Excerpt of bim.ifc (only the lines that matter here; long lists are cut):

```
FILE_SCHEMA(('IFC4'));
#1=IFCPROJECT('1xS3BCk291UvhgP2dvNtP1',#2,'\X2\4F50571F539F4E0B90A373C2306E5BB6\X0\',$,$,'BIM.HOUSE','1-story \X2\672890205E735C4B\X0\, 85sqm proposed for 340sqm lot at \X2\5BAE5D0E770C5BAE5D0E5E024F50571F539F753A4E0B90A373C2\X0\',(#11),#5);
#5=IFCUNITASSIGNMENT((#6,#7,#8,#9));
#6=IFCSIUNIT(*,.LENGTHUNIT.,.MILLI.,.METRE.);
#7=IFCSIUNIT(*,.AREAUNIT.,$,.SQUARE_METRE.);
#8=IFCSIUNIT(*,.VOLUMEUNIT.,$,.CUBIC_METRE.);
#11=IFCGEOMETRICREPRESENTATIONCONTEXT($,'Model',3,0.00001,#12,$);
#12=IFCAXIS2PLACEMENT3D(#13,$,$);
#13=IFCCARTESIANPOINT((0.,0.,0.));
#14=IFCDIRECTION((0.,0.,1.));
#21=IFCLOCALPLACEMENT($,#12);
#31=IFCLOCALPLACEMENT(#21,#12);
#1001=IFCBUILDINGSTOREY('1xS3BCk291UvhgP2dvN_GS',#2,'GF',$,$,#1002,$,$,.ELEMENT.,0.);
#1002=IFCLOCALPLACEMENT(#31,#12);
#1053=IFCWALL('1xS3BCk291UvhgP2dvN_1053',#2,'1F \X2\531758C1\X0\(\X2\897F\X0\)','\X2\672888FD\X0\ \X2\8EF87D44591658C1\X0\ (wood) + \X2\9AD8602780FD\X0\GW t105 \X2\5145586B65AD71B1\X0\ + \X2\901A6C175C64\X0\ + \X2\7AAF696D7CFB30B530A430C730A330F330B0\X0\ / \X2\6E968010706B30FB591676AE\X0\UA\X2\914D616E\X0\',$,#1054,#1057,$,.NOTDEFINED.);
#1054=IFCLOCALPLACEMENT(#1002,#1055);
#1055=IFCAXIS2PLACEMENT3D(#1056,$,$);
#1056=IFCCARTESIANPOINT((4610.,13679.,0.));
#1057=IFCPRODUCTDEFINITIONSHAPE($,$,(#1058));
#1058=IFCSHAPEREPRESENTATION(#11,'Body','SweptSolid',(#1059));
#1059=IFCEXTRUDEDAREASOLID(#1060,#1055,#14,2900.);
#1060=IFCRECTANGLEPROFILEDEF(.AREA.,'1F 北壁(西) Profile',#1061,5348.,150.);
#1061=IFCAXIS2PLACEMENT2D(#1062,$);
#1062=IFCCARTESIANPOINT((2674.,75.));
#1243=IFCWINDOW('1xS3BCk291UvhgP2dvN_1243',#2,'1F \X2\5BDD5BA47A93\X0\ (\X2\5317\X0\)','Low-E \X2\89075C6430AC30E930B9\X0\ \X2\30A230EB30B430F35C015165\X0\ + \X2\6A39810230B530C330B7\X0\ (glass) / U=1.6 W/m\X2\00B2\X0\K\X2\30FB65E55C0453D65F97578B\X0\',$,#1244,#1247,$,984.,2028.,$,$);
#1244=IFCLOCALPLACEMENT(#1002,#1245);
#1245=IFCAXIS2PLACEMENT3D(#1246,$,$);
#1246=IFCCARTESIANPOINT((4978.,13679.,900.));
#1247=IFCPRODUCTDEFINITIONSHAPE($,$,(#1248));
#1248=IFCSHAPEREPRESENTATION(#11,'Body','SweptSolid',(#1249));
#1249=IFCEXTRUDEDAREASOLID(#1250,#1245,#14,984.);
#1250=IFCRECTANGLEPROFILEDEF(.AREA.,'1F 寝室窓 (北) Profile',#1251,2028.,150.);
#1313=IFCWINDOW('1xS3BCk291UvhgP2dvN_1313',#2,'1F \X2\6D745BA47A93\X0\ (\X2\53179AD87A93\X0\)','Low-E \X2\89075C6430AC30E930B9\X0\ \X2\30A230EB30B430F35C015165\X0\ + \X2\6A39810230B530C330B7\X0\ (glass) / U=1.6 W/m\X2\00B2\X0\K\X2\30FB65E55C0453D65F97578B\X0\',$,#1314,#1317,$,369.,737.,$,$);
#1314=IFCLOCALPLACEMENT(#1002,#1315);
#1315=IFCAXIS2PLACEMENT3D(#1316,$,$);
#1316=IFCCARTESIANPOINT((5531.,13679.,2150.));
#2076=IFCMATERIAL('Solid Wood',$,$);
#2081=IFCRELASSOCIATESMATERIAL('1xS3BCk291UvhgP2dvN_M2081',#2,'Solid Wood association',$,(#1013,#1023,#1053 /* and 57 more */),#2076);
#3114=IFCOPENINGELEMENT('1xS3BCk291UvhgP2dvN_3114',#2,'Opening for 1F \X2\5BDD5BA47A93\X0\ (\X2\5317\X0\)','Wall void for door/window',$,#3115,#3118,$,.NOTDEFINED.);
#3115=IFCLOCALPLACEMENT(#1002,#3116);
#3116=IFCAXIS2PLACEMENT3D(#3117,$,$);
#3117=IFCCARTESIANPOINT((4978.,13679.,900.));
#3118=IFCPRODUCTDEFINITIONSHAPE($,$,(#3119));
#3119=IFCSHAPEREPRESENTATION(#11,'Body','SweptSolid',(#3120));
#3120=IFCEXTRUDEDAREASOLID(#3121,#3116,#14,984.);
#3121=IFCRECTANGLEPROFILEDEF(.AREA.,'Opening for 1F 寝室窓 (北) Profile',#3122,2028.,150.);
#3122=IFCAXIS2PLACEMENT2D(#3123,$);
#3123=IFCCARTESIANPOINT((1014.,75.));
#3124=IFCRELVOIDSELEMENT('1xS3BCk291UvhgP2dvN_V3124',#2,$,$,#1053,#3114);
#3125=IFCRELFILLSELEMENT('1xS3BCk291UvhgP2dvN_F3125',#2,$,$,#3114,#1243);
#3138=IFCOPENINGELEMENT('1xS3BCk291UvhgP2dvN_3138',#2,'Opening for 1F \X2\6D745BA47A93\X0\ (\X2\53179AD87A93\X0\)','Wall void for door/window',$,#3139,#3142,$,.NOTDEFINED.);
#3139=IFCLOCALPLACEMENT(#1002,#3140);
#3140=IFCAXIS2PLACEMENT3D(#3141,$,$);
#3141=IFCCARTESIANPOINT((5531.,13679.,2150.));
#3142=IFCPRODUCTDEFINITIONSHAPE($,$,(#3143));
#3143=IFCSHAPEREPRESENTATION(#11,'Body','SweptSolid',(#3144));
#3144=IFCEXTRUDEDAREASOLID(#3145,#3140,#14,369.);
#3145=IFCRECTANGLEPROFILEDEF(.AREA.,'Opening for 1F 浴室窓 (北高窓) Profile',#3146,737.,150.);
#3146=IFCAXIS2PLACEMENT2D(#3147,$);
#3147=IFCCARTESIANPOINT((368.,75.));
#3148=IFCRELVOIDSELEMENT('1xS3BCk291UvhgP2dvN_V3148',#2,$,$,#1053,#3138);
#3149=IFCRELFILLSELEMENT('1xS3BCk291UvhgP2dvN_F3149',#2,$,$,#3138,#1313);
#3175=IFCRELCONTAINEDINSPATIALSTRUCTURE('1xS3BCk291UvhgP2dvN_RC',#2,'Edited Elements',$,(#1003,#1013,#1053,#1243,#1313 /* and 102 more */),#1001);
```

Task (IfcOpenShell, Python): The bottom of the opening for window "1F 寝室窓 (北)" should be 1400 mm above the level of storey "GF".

```python
import numpy as np
import ifcopenshell
import ifcopenshell.api.geometry
import ifcopenshell.geom
import ifcopenshell.util.element
import ifcopenshell.util.placement
import ifcopenshell.util.shape
import ifcopenshell.util.unit

model = ifcopenshell.open("bim.ifc")
unit_scale = ifcopenshell.util.unit.calculate_unit_scale(model)

window = model.by_id(1243)
opening = window.FillsVoids[0].RelatingOpeningElement
storey = ifcopenshell.util.element.get_container(window, ifc_class="IfcBuildingStorey")
level = ifcopenshell.util.placement.get_local_placement(storey.ObjectPlacement)[2, 3]

# The opening's origin need not be at the sill, so measure its lowest point.
shape = ifcopenshell.geom.create_shape(ifcopenshell.geom.settings(), opening)
bottom = ifcopenshell.util.shape.get_shape_bottom_elevation(shape, shape.geometry) / unit_scale
dz = level + 1400.0 - bottom

shift = np.array([0.0, 0.0, dz])
# The window is not placed relative to its opening, so move both.
for product in (opening, window):
    matrix = ifcopenshell.util.placement.get_local_placement(product.ObjectPlacement)
    matrix[:3, 3] += shift
    ifcopenshell.api.geometry.edit_object_placement(model, product=product, matrix=matrix, is_si=False)

print(f"moved by {dz * unit_scale:+.3f} m")

model.write("bim_edited.ifc")
```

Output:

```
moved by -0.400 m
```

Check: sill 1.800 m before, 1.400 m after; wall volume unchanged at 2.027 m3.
